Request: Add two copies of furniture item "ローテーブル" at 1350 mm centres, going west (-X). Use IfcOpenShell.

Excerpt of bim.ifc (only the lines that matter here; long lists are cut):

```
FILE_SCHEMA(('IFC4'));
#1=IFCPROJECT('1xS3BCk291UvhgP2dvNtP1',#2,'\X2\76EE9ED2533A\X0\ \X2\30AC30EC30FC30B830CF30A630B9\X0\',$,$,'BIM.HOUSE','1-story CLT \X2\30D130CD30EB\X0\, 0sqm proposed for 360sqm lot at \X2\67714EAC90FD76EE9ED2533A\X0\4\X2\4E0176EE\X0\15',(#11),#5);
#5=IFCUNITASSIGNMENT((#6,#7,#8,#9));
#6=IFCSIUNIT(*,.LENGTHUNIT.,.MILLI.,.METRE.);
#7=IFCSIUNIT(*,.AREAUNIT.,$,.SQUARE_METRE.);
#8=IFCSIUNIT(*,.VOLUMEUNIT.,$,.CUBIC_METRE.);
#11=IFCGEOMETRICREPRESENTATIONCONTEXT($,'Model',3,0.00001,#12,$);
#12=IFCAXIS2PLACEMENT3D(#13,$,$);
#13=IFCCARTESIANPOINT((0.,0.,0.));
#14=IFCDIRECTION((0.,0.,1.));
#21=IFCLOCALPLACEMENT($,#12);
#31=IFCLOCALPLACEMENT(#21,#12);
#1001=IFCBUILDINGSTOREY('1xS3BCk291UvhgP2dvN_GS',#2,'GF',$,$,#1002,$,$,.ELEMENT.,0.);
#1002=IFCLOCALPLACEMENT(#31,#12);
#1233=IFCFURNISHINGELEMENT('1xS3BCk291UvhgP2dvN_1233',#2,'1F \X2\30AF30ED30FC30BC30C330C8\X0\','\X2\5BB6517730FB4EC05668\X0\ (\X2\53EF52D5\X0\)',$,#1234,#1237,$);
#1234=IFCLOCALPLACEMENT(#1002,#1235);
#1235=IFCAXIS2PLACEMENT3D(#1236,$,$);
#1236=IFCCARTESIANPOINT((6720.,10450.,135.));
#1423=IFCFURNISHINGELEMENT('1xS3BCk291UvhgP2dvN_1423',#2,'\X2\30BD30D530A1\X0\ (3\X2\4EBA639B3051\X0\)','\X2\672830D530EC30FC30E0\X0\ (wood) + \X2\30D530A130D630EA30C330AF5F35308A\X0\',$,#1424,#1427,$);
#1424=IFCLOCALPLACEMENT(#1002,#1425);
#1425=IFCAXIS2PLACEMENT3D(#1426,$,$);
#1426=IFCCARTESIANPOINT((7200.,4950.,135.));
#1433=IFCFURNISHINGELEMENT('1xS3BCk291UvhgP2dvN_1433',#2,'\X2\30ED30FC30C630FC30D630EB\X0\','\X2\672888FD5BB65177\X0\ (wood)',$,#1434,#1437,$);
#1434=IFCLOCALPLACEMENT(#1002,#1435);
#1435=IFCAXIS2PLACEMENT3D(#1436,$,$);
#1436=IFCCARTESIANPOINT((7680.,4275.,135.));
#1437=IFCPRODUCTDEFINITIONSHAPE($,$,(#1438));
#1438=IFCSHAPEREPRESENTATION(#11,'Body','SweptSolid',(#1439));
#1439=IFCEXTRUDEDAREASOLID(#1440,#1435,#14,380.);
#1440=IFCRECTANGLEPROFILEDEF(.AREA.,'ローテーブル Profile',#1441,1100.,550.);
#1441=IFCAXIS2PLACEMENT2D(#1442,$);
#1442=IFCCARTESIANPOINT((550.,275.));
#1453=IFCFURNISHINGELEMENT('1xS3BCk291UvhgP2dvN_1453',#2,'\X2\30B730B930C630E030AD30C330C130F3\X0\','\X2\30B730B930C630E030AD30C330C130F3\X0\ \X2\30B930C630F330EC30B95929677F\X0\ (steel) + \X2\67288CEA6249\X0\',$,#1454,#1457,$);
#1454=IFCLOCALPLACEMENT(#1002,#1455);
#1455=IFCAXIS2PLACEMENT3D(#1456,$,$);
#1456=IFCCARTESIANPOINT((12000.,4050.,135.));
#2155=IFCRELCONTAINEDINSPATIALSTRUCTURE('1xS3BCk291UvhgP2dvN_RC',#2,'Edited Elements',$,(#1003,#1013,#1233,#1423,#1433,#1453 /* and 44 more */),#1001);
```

```python
import numpy as np
import ifcopenshell
import ifcopenshell.api.geometry
import ifcopenshell.api.root
import ifcopenshell.util.element
import ifcopenshell.util.placement

model = ifcopenshell.open("bim.ifc")


def reuse_history(source, copy):
    """copy_class also copies each property set's owner history, people and application; keep the originals."""
    for rel in copy.IsDefinedBy:
        if rel.is_a("IfcRelDefinesByProperties") and (history := rel.RelatingPropertyDefinition.OwnerHistory):
            rel.RelatingPropertyDefinition.OwnerHistory = source.OwnerHistory
            ifcopenshell.util.element.remove_deep2(model, history)


source = model.by_guid("1xS3BCk291UvhgP2dvN_1433")
base = ifcopenshell.util.placement.get_local_placement(source.ObjectPlacement)
step = np.array([-1.0, 0.0, 0.0]) * 1350.0

for i in range(1, 3):
    copy = ifcopenshell.api.root.copy_class(model, product=source)
    copy.Representation = ifcopenshell.util.element.copy_deep(
        model, source.Representation, exclude=["IfcGeometricRepresentationContext", "IfcRepresentationMap"]
    )
    reuse_history(source, copy)
    matrix = base.copy()
    matrix[:3, 3] += i * step
    print("added at", matrix[:3, 3].round(3) + 0.0)
    ifcopenshell.api.geometry.edit_object_placement(model, product=copy, matrix=matrix, is_si=False)

model.write("bim_rev.ifc")
```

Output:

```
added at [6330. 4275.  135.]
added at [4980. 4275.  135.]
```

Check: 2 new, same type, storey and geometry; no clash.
